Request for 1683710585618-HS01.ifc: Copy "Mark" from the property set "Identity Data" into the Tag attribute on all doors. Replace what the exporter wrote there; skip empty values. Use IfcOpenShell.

First a look at what the model holds.

```python
import ifcopenshell
import ifcopenshell.util.element

model = ifcopenshell.open("1683710585618-HS01.ifc")
print(model.schema)
doors = model.by_type("IfcDoor")
print(len(doors), "doors")
for e in doors[:8]:
    source = ifcopenshell.util.element.get_pset(e, "Identity Data", "Mark")
    target = e.Tag
    print(e.id(), repr(source), repr(target), sep=" | ")
```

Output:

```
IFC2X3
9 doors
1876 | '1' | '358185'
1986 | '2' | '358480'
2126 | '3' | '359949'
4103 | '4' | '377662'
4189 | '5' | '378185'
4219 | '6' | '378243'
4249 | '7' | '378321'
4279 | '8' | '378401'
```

```python
import ifcopenshell
import ifcopenshell.util.element

model = ifcopenshell.open("1683710585618-HS01.ifc")

count = 0
for e in model.by_type("IfcDoor"):
    value = ifcopenshell.util.element.get_pset(e, "Identity Data", "Mark")
    current = e.Tag
    if not value or not value.strip() or current == value:
        continue
    e.Tag = value
    count += 1

print(count, "doors updated")

model.write("1683710585618-HS01_updated.ifc")
```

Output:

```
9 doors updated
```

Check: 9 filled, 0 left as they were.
